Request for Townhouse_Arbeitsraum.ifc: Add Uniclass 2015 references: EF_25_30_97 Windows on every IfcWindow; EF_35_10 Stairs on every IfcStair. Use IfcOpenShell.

First a look at what the model holds.

```python
import ifcopenshell

model = ifcopenshell.open("Townhouse_Arbeitsraum.ifc")
print(model.schema)
print("classifications:", [c.Name for c in model.by_type("IfcClassification")])
for ifc_class in ("IfcDoor", "IfcRoof", "IfcStair", "IfcWall", "IfcWindow"):
    print(ifc_class, len(model.by_type(ifc_class)))
```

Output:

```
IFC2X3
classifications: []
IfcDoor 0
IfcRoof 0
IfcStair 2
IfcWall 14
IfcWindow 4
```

```python
import ifcopenshell
import ifcopenshell.api.classification

model = ifcopenshell.open("Townhouse_Arbeitsraum.ifc")

# IFC2X3 requires Source and Edition and has no link from the project to the system.
system = model.create_entity("IfcClassification", Source="NBS", Edition="2015", Name="Uniclass 2015")

codes = {
    "IfcWindow": ("EF_25_30_97", "Windows"),
    "IfcStair": ("EF_35_10", "Stairs"),
}
for ifc_class, (code, name) in codes.items():
    products = model.by_type(ifc_class)
    ifcopenshell.api.classification.add_reference(
        model, products=products, classification=system, identification=code, name=name
    )
    print(code, len(products))

model.write("Townhouse_Arbeitsraum_edited.ifc")
```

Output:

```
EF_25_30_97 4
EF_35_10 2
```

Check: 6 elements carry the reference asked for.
